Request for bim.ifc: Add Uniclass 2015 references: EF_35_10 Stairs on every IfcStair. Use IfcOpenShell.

First a look at what the model holds.

```python
import ifcopenshell

model = ifcopenshell.open("bim.ifc")
print(model.schema)
print("classifications:", [c.Name for c in model.by_type("IfcClassification")])
for ifc_class in ("IfcDoor", "IfcRoof", "IfcStair", "IfcWall", "IfcWindow"):
    print(ifc_class, len(model.by_type(ifc_class)))
```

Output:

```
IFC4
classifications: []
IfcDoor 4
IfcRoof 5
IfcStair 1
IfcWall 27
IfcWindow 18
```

```python
import ifcopenshell
import ifcopenshell.api.classification

model = ifcopenshell.open("bim.ifc")

system = ifcopenshell.api.classification.add_classification(model, classification="Uniclass 2015")

codes = {
    "IfcStair": ("EF_35_10", "Stairs"),
}
for ifc_class, (code, name) in codes.items():
    products = model.by_type(ifc_class)
    ifcopenshell.api.classification.add_reference(
        model, products=products, classification=system, identification=code, name=name
    )
    print(code, len(products))

model.write("bim_rev.ifc")
```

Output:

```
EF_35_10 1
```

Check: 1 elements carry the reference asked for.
